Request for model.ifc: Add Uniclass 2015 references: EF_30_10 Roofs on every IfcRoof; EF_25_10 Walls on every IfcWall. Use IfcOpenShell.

First a look at what the model holds.

```python
import ifcopenshell

model = ifcopenshell.open("model.ifc")
print(model.schema)
print("classifications:", [c.Name for c in model.by_type("IfcClassification")])
for ifc_class in ("IfcDoor", "IfcRoof", "IfcStair", "IfcWall", "IfcWindow"):
    print(ifc_class, len(model.by_type(ifc_class)))
```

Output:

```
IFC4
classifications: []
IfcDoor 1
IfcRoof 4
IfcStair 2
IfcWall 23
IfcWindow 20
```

```python
import ifcopenshell
import ifcopenshell.api.classification

model = ifcopenshell.open("model.ifc")

system = ifcopenshell.api.classification.add_classification(model, classification="Uniclass 2015")

codes = {
    "IfcRoof": ("EF_30_10", "Roofs"),
    "IfcWall": ("EF_25_10", "Walls"),
}
for ifc_class, (code, name) in codes.items():
    products = model.by_type(ifc_class)
    ifcopenshell.api.classification.add_reference(
        model, products=products, classification=system, identification=code, name=name
    )
    print(code, len(products))

model.write("model_rev.ifc")
```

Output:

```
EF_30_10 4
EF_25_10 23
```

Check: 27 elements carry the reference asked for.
